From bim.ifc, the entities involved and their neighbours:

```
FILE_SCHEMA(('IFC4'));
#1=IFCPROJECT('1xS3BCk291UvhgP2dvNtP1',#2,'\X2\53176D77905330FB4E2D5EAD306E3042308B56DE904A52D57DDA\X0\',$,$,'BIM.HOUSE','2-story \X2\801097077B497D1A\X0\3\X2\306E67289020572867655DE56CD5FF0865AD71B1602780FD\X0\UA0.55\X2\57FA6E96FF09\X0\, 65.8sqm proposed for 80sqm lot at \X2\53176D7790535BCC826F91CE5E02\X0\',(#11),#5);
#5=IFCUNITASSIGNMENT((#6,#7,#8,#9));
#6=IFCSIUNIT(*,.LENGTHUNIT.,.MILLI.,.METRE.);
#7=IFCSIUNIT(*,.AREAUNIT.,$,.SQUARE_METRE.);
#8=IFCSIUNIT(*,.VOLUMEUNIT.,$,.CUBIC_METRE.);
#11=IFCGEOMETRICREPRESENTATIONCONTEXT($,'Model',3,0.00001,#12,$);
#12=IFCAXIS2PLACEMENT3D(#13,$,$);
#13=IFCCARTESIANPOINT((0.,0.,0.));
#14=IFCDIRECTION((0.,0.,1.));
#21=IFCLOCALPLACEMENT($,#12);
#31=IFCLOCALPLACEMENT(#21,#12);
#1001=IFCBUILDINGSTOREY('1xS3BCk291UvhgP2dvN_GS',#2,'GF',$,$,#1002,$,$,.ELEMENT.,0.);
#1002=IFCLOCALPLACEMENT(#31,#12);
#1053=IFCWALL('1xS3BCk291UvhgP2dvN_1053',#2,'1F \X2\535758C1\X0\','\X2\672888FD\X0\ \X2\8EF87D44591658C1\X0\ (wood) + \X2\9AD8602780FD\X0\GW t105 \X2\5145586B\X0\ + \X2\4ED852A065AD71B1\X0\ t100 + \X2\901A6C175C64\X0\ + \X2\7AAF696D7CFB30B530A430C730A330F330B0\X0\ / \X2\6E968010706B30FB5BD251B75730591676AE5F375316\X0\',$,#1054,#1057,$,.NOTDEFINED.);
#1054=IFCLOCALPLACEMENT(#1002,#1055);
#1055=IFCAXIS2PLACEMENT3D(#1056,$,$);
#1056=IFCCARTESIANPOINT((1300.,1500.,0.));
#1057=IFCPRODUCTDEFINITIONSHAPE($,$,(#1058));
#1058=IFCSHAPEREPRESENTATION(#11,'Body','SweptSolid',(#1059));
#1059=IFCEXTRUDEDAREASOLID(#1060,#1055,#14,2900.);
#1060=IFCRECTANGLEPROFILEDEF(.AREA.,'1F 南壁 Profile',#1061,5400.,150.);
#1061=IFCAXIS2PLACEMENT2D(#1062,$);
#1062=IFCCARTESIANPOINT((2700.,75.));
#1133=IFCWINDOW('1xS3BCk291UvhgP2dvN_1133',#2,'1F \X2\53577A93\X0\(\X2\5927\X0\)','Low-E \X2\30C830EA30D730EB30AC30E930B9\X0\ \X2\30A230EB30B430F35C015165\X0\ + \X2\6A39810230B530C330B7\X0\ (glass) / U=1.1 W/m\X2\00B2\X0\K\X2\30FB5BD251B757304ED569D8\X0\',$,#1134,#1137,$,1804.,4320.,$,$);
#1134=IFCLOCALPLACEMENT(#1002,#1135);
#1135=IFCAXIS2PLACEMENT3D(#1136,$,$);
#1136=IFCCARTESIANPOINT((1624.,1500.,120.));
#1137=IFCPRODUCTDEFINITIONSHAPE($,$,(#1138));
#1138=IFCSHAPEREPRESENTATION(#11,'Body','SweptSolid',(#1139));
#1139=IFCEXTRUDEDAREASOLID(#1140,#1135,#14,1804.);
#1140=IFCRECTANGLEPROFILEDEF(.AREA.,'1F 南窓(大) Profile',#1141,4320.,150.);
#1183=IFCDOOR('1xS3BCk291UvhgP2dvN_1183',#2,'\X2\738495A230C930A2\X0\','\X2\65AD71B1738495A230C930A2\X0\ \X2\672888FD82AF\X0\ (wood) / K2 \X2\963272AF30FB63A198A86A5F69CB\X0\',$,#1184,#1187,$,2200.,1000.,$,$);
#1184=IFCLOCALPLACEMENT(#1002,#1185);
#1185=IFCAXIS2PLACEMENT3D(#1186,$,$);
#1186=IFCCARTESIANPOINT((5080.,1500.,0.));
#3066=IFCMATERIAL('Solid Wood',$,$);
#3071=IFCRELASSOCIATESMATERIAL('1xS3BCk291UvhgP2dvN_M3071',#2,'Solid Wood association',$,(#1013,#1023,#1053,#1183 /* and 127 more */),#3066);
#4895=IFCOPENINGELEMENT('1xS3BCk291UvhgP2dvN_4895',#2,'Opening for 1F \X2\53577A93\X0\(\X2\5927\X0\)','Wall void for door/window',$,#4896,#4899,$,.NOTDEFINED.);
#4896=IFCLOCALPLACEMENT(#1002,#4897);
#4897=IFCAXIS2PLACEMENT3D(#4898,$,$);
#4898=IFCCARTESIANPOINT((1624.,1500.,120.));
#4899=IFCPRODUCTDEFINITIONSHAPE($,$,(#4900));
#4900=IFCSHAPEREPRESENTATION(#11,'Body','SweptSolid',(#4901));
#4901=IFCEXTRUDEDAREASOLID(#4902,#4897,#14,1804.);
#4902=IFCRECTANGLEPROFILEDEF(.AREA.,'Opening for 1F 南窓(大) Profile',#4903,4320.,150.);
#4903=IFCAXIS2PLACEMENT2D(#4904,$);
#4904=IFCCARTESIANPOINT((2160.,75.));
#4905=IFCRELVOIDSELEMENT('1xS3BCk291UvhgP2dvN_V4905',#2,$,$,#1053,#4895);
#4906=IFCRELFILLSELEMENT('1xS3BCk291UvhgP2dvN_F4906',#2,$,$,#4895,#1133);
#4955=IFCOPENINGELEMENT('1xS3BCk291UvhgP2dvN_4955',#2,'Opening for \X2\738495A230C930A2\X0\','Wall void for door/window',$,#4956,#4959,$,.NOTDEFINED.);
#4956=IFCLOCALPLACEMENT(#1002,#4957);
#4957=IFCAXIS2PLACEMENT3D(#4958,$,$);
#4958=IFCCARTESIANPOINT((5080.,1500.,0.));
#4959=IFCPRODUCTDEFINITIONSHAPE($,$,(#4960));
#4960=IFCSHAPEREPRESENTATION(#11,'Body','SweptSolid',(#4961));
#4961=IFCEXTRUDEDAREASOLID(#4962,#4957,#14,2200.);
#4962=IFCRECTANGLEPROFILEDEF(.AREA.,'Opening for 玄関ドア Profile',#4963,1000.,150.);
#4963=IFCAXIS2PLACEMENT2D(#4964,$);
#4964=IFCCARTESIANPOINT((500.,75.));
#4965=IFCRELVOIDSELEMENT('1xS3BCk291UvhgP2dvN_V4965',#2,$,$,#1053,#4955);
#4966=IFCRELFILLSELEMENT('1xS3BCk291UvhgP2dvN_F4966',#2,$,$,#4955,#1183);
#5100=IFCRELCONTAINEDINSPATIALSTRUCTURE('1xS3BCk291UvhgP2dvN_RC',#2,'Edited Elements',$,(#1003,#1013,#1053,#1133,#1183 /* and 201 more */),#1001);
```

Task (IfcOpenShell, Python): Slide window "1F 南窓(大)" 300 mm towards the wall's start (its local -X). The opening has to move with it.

```python
import ifcopenshell
import ifcopenshell.api.geometry
import ifcopenshell.util.placement
import ifcopenshell.util.unit

model = ifcopenshell.open("bim.ifc")
unit_scale = ifcopenshell.util.unit.calculate_unit_scale(model)

window = model.by_guid("1xS3BCk291UvhgP2dvN_1133")
opening = window.FillsVoids[0].RelatingOpeningElement
wall = opening.VoidsElements[0].RelatingBuildingElement

wall_matrix = ifcopenshell.util.placement.get_local_placement(wall.ObjectPlacement)
shift = wall_matrix[:3, 0] * -0.3 / unit_scale
before = ifcopenshell.util.placement.get_local_placement(window.ObjectPlacement)[:3, 3].copy()

# The window is not placed relative to its opening, so move both.
for product in (opening, window):
    matrix = ifcopenshell.util.placement.get_local_placement(product.ObjectPlacement)
    matrix[:3, 3] += shift
    ifcopenshell.api.geometry.edit_object_placement(model, product=product, matrix=matrix, is_si=False)

after = ifcopenshell.util.placement.get_local_placement(window.ObjectPlacement)[:3, 3]
print("window moved by", (after - before).round(3) + 0.0)

model.write("bim_rev.ifc")
```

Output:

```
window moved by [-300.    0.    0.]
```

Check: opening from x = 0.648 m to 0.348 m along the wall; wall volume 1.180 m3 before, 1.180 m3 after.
